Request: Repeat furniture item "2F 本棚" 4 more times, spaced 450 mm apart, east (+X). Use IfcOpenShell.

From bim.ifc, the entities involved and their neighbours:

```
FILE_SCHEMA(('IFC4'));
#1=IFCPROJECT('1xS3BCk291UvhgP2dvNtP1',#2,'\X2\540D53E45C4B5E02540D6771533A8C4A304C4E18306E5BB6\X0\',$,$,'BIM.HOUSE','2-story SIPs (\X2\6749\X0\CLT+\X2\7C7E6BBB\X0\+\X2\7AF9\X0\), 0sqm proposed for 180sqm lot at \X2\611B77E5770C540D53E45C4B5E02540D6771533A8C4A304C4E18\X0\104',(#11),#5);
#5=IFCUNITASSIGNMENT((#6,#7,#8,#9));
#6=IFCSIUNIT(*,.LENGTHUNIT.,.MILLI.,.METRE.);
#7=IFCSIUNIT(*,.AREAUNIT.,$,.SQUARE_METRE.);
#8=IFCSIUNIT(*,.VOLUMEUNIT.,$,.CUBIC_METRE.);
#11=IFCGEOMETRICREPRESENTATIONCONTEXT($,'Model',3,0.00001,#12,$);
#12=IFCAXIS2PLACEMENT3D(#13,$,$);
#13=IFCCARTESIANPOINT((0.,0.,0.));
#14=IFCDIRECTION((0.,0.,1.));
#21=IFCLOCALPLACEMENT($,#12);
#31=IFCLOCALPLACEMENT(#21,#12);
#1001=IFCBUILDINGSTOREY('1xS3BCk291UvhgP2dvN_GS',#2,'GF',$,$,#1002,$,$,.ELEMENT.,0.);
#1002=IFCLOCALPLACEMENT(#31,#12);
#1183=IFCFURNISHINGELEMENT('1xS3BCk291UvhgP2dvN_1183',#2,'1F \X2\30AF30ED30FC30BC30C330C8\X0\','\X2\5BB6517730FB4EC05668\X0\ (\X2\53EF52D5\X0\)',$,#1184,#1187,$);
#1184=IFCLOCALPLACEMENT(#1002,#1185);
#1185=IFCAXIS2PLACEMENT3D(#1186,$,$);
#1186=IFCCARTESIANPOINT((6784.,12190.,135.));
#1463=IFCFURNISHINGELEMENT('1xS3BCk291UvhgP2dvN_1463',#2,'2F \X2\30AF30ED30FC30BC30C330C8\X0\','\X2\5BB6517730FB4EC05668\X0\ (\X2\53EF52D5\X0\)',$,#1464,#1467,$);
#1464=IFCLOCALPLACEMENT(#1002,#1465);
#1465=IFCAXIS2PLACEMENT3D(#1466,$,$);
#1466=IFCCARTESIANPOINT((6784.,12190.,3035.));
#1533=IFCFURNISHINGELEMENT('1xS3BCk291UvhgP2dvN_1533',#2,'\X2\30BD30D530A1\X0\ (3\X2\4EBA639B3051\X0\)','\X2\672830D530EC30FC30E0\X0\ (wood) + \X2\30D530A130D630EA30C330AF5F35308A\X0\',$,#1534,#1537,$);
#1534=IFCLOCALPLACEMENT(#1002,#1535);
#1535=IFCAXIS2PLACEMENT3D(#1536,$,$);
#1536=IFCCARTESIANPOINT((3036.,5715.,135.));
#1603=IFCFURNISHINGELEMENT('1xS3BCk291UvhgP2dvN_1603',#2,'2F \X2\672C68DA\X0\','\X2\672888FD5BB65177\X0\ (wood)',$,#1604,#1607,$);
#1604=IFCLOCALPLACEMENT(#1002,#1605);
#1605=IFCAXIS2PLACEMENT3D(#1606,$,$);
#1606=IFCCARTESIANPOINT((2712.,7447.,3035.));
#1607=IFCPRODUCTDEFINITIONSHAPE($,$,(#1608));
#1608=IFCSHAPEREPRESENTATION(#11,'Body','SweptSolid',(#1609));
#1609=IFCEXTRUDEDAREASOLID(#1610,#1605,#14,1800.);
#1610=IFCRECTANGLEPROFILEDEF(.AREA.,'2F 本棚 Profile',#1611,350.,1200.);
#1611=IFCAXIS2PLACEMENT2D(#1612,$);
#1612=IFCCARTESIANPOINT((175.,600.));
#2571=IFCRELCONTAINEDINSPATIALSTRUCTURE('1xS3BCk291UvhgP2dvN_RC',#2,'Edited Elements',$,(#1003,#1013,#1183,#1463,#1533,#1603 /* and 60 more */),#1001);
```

```python
import numpy as np
import ifcopenshell
import ifcopenshell.api.geometry
import ifcopenshell.api.root
import ifcopenshell.util.element
import ifcopenshell.util.placement

model = ifcopenshell.open("bim.ifc")


def reuse_history(source, copy):
    """copy_class also copies each property set's owner history, people and application; keep the originals."""
    for rel in copy.IsDefinedBy:
        if rel.is_a("IfcRelDefinesByProperties") and (history := rel.RelatingPropertyDefinition.OwnerHistory):
            rel.RelatingPropertyDefinition.OwnerHistory = source.OwnerHistory
            ifcopenshell.util.element.remove_deep2(model, history)


source = model.by_id(1603)
base = ifcopenshell.util.placement.get_local_placement(source.ObjectPlacement)
step = np.array([1.0, 0.0, 0.0]) * 450.0

for i in range(1, 5):
    copy = ifcopenshell.api.root.copy_class(model, product=source)
    copy.Representation = ifcopenshell.util.element.copy_deep(
        model, source.Representation, exclude=["IfcGeometricRepresentationContext", "IfcRepresentationMap"]
    )
    reuse_history(source, copy)
    matrix = base.copy()
    matrix[:3, 3] += i * step
    print("added at", matrix[:3, 3].round(3) + 0.0)
    ifcopenshell.api.geometry.edit_object_placement(model, product=copy, matrix=matrix, is_si=False)

model.write("bim-out.ifc")
```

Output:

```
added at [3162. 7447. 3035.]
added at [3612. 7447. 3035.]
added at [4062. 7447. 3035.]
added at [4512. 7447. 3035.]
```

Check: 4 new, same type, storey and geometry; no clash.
